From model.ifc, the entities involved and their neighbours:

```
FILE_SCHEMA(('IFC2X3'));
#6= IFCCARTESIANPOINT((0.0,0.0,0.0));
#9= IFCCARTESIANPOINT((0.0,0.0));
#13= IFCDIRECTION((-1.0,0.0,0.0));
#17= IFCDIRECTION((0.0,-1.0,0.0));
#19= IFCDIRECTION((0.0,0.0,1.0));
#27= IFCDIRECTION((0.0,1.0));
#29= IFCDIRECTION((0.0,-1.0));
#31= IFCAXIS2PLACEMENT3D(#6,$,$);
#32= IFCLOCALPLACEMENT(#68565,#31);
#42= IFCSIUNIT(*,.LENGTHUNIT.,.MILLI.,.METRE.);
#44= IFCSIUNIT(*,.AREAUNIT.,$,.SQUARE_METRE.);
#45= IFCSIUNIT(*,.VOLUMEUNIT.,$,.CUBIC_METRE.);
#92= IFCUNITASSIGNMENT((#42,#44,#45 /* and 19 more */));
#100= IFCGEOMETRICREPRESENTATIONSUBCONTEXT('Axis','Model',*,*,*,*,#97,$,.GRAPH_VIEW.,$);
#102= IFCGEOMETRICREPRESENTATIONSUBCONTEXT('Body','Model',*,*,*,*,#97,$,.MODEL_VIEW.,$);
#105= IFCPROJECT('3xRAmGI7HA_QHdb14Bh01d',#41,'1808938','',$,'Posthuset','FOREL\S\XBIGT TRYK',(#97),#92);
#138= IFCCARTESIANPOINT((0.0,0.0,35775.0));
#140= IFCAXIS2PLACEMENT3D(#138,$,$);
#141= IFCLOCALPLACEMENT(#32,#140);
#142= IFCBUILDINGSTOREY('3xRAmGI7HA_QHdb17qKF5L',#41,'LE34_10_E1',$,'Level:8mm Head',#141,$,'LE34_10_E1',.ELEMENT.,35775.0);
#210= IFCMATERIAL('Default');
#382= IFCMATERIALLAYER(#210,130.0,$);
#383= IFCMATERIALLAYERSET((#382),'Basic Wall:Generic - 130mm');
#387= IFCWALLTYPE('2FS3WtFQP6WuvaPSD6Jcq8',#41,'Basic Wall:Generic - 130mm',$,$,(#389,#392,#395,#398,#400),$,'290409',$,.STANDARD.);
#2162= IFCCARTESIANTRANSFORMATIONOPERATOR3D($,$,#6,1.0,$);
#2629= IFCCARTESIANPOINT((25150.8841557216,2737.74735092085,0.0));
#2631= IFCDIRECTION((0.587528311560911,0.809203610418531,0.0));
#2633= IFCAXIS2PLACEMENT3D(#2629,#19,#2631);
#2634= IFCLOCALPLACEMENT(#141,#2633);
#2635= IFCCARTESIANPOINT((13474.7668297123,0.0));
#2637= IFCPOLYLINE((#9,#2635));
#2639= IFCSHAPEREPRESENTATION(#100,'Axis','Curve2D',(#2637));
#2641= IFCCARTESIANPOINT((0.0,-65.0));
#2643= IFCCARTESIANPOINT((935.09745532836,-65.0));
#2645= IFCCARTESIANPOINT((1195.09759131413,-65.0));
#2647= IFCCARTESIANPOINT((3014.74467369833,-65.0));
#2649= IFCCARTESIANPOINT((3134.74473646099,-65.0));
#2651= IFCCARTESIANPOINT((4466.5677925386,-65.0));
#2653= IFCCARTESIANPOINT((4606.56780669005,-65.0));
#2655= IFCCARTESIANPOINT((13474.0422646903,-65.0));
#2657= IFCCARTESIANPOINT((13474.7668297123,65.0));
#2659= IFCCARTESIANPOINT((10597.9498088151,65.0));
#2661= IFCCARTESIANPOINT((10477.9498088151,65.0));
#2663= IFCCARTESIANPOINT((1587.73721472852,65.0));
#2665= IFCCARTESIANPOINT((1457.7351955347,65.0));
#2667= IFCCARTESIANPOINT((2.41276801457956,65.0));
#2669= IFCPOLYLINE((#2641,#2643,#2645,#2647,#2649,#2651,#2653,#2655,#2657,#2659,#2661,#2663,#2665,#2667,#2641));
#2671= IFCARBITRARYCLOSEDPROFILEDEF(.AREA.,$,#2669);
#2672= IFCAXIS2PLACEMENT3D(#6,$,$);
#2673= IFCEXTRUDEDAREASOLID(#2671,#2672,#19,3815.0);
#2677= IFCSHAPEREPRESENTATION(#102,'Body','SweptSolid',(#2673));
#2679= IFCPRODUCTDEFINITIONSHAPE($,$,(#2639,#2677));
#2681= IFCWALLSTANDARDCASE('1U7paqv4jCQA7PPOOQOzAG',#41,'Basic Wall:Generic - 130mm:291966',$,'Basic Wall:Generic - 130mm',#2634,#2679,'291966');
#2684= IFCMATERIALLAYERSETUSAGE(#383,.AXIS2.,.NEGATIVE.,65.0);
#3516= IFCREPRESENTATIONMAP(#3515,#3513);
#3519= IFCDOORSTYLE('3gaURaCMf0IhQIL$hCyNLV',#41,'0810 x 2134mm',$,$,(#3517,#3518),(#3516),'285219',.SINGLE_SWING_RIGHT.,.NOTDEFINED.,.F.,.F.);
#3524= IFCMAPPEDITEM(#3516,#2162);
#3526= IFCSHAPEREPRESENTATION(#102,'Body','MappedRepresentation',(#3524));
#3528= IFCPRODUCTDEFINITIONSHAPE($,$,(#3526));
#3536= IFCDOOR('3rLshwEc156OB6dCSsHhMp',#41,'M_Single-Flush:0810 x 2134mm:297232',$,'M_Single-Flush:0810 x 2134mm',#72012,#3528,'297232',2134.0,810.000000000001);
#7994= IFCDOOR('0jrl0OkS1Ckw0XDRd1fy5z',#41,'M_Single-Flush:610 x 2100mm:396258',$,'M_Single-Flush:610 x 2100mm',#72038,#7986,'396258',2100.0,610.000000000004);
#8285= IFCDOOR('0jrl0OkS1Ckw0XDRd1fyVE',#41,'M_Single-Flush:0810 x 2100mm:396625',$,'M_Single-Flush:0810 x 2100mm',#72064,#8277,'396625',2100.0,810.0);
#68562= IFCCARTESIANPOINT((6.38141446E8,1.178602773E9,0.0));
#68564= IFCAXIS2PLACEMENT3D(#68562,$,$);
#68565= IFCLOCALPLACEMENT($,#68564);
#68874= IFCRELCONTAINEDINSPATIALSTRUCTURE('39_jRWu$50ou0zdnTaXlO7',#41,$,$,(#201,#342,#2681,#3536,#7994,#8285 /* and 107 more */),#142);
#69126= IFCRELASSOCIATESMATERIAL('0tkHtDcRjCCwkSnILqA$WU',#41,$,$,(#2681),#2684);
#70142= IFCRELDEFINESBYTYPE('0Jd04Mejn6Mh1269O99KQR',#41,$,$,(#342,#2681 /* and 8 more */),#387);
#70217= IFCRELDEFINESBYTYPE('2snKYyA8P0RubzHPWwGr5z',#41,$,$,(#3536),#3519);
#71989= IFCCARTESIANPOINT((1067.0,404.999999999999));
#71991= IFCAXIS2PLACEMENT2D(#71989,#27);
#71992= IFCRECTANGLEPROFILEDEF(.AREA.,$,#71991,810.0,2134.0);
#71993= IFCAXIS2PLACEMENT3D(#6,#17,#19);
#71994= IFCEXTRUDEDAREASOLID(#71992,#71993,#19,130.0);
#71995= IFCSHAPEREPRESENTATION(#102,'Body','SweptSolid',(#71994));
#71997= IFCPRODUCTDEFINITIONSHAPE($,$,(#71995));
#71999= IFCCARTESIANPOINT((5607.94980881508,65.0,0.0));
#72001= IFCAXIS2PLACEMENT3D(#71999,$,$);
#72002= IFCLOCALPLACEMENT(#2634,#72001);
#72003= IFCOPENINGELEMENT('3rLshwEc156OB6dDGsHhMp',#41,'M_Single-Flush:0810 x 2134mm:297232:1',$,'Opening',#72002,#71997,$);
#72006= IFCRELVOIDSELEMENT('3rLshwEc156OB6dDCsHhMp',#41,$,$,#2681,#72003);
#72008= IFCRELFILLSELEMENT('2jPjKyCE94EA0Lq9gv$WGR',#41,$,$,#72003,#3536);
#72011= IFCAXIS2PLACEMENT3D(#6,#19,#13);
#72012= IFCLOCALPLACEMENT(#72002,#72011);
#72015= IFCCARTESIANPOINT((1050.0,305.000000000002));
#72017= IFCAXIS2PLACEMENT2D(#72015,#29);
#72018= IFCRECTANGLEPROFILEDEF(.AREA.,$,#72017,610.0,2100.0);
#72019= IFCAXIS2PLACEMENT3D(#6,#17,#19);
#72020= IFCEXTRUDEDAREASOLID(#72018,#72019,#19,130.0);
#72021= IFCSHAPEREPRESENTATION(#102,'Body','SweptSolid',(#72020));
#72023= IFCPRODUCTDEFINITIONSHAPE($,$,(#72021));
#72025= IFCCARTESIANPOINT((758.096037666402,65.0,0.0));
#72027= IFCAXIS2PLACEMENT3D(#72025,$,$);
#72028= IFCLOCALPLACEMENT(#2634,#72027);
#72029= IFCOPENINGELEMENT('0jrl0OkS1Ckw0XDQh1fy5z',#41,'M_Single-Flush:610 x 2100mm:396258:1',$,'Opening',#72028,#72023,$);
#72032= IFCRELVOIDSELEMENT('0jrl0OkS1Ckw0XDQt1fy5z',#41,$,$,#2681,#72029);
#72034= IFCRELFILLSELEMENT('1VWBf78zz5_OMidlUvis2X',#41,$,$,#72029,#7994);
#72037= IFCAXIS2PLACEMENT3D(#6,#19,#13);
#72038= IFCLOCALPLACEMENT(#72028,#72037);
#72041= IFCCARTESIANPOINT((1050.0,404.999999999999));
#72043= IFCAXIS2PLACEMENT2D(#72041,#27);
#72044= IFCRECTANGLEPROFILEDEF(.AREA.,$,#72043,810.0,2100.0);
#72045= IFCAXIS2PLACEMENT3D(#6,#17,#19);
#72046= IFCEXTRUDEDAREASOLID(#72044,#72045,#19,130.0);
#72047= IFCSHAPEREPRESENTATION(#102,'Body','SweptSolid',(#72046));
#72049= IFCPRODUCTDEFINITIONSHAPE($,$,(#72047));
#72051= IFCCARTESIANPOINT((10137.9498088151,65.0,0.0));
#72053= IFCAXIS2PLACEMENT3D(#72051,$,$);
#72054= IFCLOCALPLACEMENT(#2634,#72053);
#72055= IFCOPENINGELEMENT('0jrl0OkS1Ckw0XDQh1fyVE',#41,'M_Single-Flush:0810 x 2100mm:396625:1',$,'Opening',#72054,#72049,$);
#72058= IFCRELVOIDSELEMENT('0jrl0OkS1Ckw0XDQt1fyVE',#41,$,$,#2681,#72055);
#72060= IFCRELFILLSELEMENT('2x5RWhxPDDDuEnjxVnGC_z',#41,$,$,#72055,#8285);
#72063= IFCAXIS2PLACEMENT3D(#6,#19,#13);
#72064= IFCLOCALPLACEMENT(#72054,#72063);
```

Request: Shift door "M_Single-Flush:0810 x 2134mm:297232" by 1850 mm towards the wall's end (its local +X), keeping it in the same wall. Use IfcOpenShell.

```python
import ifcopenshell
import ifcopenshell.api.geometry
import ifcopenshell.util.placement
import ifcopenshell.util.unit

model = ifcopenshell.open("model.ifc")
unit_scale = ifcopenshell.util.unit.calculate_unit_scale(model)

door = model.by_guid("3rLshwEc156OB6dCSsHhMp")
opening = door.FillsVoids[0].RelatingOpeningElement
wall = opening.VoidsElements[0].RelatingBuildingElement

wall_matrix = ifcopenshell.util.placement.get_local_placement(wall.ObjectPlacement)
shift = wall_matrix[:3, 0] * 1.85 / unit_scale
before = ifcopenshell.util.placement.get_local_placement(door.ObjectPlacement)[:3, 3].copy()

# The door is placed relative to its opening, so it follows when the opening moves.
matrix = ifcopenshell.util.placement.get_local_placement(opening.ObjectPlacement)
matrix[:3, 3] += shift
ifcopenshell.api.geometry.edit_object_placement(
    model, product=opening, matrix=matrix, is_si=False, should_transform_children=True
)

after = ifcopenshell.util.placement.get_local_placement(door.ObjectPlacement)[:3, 3]
print("door moved by", (after - before).round(3) + 0.0)

model.write("model_edited.ifc")
```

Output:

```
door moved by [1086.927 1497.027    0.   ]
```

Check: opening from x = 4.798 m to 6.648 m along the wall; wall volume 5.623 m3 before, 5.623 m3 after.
